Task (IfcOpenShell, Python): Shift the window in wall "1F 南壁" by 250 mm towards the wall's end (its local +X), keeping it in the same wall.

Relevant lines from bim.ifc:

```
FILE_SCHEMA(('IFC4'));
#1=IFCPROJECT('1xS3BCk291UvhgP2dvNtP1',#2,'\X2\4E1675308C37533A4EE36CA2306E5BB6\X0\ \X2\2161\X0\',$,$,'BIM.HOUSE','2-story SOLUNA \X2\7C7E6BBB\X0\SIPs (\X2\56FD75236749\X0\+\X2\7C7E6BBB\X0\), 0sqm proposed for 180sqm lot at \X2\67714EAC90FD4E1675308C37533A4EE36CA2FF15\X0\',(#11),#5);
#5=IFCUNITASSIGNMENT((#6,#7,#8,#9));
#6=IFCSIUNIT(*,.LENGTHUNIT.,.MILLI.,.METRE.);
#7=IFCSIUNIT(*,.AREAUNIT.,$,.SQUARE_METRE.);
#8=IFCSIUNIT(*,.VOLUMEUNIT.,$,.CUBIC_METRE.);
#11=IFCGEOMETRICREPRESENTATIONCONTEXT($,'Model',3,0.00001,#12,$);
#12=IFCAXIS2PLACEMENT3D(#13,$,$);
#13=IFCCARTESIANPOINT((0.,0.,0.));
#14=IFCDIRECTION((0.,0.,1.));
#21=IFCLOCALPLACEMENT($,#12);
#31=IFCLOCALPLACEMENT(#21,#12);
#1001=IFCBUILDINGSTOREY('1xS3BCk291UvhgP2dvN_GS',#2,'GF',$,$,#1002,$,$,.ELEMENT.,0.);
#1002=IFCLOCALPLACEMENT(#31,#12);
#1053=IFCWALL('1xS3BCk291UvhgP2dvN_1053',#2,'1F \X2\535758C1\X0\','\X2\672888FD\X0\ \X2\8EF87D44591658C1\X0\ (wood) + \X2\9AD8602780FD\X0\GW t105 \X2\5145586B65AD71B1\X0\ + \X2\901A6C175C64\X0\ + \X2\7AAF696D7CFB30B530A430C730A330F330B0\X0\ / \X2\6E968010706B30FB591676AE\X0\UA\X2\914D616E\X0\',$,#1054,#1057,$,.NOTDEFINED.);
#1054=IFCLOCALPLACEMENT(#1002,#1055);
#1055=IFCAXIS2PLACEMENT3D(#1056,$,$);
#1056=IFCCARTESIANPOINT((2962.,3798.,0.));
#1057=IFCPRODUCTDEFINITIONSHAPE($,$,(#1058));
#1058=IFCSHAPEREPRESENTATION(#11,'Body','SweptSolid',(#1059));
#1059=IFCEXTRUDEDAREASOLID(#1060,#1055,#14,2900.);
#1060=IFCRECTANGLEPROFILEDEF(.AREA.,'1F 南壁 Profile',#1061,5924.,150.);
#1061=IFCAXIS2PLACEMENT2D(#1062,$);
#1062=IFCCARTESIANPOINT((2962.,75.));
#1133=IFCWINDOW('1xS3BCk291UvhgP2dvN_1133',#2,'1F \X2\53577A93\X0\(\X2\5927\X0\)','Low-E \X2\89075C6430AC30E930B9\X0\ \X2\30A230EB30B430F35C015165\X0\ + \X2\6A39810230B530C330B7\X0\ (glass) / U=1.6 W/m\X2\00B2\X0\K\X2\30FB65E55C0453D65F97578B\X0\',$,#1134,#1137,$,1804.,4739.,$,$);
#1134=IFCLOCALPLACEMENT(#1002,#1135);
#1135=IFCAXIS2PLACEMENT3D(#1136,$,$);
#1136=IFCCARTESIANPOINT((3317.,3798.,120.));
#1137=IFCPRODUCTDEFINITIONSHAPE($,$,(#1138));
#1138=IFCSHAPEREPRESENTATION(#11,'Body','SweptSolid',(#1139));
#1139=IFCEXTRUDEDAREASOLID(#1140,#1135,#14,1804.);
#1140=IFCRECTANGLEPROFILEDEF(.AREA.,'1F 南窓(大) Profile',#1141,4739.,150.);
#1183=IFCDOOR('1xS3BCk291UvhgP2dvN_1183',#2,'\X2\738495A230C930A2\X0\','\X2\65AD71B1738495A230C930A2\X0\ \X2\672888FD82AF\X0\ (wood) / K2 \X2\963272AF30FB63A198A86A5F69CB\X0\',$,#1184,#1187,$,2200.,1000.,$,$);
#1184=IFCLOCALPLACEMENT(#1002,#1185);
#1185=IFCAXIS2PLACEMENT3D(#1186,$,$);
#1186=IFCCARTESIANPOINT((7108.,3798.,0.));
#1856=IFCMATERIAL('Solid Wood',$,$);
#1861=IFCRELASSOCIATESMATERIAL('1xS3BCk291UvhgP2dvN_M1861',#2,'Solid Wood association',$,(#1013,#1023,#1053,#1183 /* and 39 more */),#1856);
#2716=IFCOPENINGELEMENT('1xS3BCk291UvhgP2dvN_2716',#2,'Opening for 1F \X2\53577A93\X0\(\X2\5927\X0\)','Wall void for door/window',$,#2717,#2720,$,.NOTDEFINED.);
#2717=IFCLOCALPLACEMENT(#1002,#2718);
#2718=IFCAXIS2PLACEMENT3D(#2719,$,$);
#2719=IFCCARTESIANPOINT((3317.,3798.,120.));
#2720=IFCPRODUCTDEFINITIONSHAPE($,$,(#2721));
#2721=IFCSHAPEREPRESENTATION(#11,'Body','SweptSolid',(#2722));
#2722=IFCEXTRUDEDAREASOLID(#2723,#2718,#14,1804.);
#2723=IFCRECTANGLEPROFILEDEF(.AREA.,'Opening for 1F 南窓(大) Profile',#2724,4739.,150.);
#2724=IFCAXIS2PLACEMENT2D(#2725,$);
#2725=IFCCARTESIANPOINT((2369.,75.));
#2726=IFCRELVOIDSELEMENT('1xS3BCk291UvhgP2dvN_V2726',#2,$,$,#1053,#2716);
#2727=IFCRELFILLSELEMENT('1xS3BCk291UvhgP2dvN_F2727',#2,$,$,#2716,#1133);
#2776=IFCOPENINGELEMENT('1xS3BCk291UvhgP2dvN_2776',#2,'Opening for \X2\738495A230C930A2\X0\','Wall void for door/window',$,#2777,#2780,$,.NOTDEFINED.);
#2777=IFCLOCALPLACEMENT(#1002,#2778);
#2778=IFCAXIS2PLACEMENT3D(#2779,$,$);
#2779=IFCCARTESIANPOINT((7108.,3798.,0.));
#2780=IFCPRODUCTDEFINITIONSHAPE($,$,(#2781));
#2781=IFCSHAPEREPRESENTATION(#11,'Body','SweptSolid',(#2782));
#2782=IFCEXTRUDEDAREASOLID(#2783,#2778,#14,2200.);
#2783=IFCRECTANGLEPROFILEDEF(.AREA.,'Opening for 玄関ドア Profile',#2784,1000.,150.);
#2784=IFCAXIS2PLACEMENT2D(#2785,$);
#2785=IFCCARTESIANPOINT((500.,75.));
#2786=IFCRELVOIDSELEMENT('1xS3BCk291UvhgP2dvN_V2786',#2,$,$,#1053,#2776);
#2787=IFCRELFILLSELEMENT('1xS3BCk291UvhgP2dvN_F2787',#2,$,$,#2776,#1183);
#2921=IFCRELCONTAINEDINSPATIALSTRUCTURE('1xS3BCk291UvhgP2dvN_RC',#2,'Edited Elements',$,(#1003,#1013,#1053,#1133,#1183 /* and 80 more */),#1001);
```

```python
import ifcopenshell
import ifcopenshell.api.geometry
import ifcopenshell.util.placement
import ifcopenshell.util.unit

model = ifcopenshell.open("bim.ifc")
unit_scale = ifcopenshell.util.unit.calculate_unit_scale(model)

window = model.by_id(1133)
opening = window.FillsVoids[0].RelatingOpeningElement
wall = opening.VoidsElements[0].RelatingBuildingElement

wall_matrix = ifcopenshell.util.placement.get_local_placement(wall.ObjectPlacement)
shift = wall_matrix[:3, 0] * 0.25 / unit_scale
before = ifcopenshell.util.placement.get_local_placement(window.ObjectPlacement)[:3, 3].copy()

# The window is not placed relative to its opening, so move both.
for product in (opening, window):
    matrix = ifcopenshell.util.placement.get_local_placement(product.ObjectPlacement)
    matrix[:3, 3] += shift
    ifcopenshell.api.geometry.edit_object_placement(model, product=product, matrix=matrix, is_si=False)

after = ifcopenshell.util.placement.get_local_placement(window.ObjectPlacement)[:3, 3]
print("window moved by", (after - before).round(3) + 0.0)

model.write("bim_edited.ifc")
```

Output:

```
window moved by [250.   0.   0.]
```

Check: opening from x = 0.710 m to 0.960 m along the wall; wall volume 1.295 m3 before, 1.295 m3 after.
